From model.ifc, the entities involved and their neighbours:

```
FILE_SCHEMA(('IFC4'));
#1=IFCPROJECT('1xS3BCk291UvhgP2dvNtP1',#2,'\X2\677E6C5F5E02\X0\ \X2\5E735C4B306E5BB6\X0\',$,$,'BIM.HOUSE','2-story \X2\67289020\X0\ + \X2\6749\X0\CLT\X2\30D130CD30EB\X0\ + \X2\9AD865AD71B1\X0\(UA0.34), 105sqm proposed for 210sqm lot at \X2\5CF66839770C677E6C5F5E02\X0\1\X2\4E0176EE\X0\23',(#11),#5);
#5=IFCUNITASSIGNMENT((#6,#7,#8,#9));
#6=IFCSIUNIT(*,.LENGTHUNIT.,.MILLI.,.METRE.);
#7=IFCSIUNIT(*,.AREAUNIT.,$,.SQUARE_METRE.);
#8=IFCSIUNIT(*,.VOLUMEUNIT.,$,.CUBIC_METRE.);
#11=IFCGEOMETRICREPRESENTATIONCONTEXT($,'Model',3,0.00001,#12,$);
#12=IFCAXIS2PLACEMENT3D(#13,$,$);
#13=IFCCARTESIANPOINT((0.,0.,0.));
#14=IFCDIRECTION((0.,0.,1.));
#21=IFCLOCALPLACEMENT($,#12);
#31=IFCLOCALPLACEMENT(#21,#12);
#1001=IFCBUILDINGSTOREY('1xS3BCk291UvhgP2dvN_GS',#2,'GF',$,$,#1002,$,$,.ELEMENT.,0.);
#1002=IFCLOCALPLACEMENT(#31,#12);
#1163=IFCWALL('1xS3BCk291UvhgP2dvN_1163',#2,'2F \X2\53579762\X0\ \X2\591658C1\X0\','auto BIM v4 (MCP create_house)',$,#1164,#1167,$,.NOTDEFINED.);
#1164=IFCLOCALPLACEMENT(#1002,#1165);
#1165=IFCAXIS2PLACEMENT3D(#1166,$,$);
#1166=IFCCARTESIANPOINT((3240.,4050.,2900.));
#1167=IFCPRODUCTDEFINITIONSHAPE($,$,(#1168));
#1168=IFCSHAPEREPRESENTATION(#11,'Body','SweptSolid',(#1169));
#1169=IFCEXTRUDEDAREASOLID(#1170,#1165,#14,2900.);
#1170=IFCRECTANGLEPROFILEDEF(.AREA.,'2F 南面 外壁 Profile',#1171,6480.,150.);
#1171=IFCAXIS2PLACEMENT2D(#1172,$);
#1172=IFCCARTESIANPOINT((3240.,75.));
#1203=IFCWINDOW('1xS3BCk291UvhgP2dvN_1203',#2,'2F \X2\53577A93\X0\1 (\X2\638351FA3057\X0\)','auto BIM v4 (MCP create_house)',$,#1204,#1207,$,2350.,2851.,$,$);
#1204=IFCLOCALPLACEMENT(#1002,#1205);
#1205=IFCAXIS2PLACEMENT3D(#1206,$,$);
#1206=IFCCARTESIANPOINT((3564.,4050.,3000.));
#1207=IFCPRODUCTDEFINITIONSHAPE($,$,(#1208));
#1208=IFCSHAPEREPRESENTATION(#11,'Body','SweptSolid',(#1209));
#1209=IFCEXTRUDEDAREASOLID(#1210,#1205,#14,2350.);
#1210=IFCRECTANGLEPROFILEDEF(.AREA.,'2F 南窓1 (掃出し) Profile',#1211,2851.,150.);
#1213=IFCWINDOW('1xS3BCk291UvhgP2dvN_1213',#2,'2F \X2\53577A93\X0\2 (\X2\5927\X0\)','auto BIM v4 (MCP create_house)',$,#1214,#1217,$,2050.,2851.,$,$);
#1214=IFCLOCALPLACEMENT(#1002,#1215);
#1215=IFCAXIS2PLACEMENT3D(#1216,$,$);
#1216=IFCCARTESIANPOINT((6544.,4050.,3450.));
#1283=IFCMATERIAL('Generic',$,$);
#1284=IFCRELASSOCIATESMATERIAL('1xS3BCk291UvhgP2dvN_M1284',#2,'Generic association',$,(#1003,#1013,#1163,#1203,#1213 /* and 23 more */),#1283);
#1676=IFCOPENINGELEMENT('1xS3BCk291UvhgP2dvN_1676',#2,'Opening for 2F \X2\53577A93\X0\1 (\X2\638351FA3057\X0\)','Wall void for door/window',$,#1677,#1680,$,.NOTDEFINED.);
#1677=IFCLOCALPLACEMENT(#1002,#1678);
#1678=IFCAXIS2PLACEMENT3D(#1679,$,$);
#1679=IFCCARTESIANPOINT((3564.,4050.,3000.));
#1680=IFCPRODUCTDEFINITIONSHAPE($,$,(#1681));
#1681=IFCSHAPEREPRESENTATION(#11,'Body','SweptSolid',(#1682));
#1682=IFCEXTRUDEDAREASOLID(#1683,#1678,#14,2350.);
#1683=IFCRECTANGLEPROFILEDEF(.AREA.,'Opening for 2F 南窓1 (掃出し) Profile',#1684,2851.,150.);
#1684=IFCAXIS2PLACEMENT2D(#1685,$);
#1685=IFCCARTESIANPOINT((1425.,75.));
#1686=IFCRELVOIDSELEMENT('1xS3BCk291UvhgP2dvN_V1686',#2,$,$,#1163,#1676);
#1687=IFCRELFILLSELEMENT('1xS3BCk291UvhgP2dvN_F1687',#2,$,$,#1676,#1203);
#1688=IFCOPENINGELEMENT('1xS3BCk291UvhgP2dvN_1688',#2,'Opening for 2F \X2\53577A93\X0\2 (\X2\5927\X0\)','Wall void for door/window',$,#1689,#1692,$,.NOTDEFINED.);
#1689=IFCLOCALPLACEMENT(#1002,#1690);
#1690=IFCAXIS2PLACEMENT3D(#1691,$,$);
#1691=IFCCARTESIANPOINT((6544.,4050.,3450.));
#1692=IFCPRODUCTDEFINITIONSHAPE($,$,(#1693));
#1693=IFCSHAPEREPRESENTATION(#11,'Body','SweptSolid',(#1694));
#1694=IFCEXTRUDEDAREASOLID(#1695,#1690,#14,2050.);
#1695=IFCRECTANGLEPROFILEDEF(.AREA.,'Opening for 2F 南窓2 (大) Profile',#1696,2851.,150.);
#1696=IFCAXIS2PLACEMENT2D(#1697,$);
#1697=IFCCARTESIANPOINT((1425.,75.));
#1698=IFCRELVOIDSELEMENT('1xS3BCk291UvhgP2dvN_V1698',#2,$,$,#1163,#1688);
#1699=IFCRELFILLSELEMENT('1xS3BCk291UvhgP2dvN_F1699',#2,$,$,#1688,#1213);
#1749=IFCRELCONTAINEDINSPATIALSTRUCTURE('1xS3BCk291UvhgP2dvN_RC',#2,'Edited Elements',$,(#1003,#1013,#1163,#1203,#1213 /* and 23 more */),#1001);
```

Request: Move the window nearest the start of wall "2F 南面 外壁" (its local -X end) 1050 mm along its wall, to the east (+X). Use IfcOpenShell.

```python
import ifcopenshell
import ifcopenshell.api.geometry
import ifcopenshell.util.placement
import ifcopenshell.util.unit

model = ifcopenshell.open("model.ifc")
unit_scale = ifcopenshell.util.unit.calculate_unit_scale(model)

window = model.by_guid("1xS3BCk291UvhgP2dvN_1203")
opening = window.FillsVoids[0].RelatingOpeningElement
wall = opening.VoidsElements[0].RelatingBuildingElement

wall_matrix = ifcopenshell.util.placement.get_local_placement(wall.ObjectPlacement)
shift = wall_matrix[:3, 0] * 1.05 / unit_scale
before = ifcopenshell.util.placement.get_local_placement(window.ObjectPlacement)[:3, 3].copy()

# The window is not placed relative to its opening, so move both.
for product in (opening, window):
    matrix = ifcopenshell.util.placement.get_local_placement(product.ObjectPlacement)
    matrix[:3, 3] += shift
    ifcopenshell.api.geometry.edit_object_placement(model, product=product, matrix=matrix, is_si=False)

after = ifcopenshell.util.placement.get_local_placement(window.ObjectPlacement)[:3, 3]
print("window moved by", (after - before).round(3) + 0.0)

model.write("model_updated.ifc")
```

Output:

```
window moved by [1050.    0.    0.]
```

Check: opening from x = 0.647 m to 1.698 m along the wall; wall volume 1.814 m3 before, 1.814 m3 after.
